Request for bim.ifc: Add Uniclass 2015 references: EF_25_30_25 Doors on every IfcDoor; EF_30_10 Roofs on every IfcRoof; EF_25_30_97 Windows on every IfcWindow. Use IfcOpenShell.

First a look at what the model holds.

```python
import ifcopenshell

model = ifcopenshell.open("bim.ifc")
print(model.schema)
print("classifications:", [c.Name for c in model.by_type("IfcClassification")])
for ifc_class in ("IfcDoor", "IfcRoof", "IfcStair", "IfcWall", "IfcWindow"):
    print(ifc_class, len(model.by_type(ifc_class)))
```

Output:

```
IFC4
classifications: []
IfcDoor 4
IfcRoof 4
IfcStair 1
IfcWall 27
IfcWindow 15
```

```python
import ifcopenshell
import ifcopenshell.api.classification

model = ifcopenshell.open("bim.ifc")

system = ifcopenshell.api.classification.add_classification(model, classification="Uniclass 2015")

codes = {
    "IfcDoor": ("EF_25_30_25", "Doors"),
    "IfcRoof": ("EF_30_10", "Roofs"),
    "IfcWindow": ("EF_25_30_97", "Windows"),
}
for ifc_class, (code, name) in codes.items():
    products = model.by_type(ifc_class)
    ifcopenshell.api.classification.add_reference(
        model, products=products, classification=system, identification=code, name=name
    )
    print(code, len(products))

model.write("bim_v2.ifc")
```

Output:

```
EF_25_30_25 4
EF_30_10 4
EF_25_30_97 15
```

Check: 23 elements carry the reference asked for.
